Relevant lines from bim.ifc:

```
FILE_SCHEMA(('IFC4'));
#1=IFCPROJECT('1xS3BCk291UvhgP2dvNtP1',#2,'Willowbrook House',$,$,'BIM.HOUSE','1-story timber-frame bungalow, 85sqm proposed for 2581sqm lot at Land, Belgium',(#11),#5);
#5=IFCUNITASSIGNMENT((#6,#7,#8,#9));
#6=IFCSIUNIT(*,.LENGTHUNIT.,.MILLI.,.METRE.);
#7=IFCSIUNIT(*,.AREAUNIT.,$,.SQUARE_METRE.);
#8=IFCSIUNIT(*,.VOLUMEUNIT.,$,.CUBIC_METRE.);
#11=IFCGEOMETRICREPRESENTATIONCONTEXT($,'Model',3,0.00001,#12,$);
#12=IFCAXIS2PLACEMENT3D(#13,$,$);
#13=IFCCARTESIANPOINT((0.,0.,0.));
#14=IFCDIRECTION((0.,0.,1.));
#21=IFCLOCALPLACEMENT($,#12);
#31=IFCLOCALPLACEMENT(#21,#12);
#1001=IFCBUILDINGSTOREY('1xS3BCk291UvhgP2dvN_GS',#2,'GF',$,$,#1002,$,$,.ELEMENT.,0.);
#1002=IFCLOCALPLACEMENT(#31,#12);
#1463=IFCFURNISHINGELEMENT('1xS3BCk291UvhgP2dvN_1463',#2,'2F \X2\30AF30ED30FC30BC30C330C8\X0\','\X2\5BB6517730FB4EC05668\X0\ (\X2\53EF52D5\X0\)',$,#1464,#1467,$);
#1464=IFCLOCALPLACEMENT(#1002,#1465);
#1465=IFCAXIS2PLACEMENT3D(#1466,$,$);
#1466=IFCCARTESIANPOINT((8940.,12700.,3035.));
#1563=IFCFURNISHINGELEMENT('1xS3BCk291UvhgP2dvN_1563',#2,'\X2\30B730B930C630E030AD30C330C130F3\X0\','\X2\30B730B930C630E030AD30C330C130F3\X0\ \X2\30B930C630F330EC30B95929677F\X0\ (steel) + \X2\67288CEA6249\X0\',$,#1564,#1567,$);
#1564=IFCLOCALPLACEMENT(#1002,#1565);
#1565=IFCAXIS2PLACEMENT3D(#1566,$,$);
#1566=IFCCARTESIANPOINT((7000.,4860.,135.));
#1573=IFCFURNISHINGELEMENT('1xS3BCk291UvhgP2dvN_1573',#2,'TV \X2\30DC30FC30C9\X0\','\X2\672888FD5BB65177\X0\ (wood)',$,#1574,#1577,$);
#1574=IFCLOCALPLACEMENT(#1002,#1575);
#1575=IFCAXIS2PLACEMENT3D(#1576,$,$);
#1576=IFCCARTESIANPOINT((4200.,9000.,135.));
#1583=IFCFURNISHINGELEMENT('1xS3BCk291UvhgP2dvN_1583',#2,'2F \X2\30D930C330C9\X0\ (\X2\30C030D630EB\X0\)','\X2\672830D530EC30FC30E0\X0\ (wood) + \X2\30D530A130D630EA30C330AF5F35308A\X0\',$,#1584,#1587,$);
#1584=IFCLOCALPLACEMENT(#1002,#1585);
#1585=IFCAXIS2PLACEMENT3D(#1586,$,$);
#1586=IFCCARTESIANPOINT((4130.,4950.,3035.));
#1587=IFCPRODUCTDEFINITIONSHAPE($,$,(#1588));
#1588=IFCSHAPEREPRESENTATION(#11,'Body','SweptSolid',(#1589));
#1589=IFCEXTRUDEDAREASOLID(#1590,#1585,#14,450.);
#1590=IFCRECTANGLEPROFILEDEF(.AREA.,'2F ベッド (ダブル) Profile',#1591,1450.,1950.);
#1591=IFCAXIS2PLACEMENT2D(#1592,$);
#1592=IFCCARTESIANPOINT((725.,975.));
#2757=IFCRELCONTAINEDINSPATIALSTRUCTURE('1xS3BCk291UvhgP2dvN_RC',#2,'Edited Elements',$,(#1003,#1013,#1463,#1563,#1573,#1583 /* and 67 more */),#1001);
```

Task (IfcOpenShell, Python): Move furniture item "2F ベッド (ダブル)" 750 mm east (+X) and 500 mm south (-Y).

```python
import ifcopenshell
import ifcopenshell.api.geometry
import ifcopenshell.util.placement

model = ifcopenshell.open("bim.ifc")

item = model.by_guid("1xS3BCk291UvhgP2dvN_1583")
matrix = ifcopenshell.util.placement.get_local_placement(item.ObjectPlacement)
matrix[0, 3] += 750.0
matrix[1, 3] -= 500.0
ifcopenshell.api.geometry.edit_object_placement(model, product=item, matrix=matrix, is_si=False)

print(ifcopenshell.util.placement.get_local_placement(item.ObjectPlacement).round(3) + 0.0)

model.write("bim_updated.ifc")
```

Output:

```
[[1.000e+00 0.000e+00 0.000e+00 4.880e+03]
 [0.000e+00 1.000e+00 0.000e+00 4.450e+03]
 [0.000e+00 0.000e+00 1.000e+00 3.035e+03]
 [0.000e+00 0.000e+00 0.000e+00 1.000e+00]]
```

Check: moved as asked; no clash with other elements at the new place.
